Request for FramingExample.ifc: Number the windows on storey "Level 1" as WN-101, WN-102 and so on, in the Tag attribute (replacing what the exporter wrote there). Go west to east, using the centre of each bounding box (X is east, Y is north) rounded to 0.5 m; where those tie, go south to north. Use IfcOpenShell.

First a look at what the model holds.

```python
import ifcopenshell
import ifcopenshell.util.element
import ifcopenshell.util.placement

model = ifcopenshell.open("FramingExample.ifc")
print(model.schema)
storey = next(s for s in model.by_type("IfcBuildingStorey") if s.Name == "Level 1")
windows = [e for e in ifcopenshell.util.element.get_decomposition(storey) if e.is_a("IfcWindow")]
for e in sorted(windows, key=lambda e: e.id()):
    origin = ifcopenshell.util.placement.get_local_placement(e.ObjectPlacement)[:3, 3]
    print(e.id(), e.Tag, e.Name, origin.round(2) + 0.0, sep=" | ")
```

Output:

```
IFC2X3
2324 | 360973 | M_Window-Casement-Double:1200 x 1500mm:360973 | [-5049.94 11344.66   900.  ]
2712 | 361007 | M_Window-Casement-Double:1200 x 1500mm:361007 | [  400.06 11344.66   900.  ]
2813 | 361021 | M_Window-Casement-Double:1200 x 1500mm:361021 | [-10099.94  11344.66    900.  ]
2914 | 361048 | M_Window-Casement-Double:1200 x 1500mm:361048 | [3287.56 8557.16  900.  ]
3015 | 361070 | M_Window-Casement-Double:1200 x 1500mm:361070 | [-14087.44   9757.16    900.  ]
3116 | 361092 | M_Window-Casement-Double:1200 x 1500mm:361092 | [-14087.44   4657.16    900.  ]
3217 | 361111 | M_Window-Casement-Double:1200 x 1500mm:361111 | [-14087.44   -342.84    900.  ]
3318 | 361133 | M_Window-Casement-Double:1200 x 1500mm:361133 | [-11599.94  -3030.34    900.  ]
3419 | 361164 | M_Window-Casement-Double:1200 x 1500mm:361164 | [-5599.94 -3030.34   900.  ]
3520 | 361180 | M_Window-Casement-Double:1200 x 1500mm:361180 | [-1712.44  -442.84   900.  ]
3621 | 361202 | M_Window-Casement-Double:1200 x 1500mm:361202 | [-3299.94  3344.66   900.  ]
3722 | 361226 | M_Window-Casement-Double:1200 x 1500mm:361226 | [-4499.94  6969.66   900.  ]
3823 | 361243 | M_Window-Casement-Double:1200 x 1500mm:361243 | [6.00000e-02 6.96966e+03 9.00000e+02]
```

```python
import ifcopenshell
import ifcopenshell.geom
import ifcopenshell.util.element
import ifcopenshell.util.shape

model = ifcopenshell.open("FramingExample.ifc")
settings = ifcopenshell.geom.settings()
settings.set("use-world-coords", True)


def centre(element):
    shape = ifcopenshell.geom.create_shape(settings, element)
    return ifcopenshell.util.shape.get_bbox_centroid(shape.geometry)


storey = next(s for s in model.by_type("IfcBuildingStorey") if s.Name == "Level 1")
windows = [e for e in ifcopenshell.util.element.get_decomposition(storey) if e.is_a("IfcWindow")]

# Insertion points can sit at a corner or the storey origin, so sort by the geometry (in metres).
centres = {e: centre(e) for e in windows}
windows.sort(key=lambda e: (round(centres[e][0] / 0.5), centres[e][1]))

for i, e in enumerate(windows, start=1):
    number = f"WN-1{i:02d}"
    e.Tag = number
    print(e.id(), number)

model.write("FramingExample-out.ifc")
```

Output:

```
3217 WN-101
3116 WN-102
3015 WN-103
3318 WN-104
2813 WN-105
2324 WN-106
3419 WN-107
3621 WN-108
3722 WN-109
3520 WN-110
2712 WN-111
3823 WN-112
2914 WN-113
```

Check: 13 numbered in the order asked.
